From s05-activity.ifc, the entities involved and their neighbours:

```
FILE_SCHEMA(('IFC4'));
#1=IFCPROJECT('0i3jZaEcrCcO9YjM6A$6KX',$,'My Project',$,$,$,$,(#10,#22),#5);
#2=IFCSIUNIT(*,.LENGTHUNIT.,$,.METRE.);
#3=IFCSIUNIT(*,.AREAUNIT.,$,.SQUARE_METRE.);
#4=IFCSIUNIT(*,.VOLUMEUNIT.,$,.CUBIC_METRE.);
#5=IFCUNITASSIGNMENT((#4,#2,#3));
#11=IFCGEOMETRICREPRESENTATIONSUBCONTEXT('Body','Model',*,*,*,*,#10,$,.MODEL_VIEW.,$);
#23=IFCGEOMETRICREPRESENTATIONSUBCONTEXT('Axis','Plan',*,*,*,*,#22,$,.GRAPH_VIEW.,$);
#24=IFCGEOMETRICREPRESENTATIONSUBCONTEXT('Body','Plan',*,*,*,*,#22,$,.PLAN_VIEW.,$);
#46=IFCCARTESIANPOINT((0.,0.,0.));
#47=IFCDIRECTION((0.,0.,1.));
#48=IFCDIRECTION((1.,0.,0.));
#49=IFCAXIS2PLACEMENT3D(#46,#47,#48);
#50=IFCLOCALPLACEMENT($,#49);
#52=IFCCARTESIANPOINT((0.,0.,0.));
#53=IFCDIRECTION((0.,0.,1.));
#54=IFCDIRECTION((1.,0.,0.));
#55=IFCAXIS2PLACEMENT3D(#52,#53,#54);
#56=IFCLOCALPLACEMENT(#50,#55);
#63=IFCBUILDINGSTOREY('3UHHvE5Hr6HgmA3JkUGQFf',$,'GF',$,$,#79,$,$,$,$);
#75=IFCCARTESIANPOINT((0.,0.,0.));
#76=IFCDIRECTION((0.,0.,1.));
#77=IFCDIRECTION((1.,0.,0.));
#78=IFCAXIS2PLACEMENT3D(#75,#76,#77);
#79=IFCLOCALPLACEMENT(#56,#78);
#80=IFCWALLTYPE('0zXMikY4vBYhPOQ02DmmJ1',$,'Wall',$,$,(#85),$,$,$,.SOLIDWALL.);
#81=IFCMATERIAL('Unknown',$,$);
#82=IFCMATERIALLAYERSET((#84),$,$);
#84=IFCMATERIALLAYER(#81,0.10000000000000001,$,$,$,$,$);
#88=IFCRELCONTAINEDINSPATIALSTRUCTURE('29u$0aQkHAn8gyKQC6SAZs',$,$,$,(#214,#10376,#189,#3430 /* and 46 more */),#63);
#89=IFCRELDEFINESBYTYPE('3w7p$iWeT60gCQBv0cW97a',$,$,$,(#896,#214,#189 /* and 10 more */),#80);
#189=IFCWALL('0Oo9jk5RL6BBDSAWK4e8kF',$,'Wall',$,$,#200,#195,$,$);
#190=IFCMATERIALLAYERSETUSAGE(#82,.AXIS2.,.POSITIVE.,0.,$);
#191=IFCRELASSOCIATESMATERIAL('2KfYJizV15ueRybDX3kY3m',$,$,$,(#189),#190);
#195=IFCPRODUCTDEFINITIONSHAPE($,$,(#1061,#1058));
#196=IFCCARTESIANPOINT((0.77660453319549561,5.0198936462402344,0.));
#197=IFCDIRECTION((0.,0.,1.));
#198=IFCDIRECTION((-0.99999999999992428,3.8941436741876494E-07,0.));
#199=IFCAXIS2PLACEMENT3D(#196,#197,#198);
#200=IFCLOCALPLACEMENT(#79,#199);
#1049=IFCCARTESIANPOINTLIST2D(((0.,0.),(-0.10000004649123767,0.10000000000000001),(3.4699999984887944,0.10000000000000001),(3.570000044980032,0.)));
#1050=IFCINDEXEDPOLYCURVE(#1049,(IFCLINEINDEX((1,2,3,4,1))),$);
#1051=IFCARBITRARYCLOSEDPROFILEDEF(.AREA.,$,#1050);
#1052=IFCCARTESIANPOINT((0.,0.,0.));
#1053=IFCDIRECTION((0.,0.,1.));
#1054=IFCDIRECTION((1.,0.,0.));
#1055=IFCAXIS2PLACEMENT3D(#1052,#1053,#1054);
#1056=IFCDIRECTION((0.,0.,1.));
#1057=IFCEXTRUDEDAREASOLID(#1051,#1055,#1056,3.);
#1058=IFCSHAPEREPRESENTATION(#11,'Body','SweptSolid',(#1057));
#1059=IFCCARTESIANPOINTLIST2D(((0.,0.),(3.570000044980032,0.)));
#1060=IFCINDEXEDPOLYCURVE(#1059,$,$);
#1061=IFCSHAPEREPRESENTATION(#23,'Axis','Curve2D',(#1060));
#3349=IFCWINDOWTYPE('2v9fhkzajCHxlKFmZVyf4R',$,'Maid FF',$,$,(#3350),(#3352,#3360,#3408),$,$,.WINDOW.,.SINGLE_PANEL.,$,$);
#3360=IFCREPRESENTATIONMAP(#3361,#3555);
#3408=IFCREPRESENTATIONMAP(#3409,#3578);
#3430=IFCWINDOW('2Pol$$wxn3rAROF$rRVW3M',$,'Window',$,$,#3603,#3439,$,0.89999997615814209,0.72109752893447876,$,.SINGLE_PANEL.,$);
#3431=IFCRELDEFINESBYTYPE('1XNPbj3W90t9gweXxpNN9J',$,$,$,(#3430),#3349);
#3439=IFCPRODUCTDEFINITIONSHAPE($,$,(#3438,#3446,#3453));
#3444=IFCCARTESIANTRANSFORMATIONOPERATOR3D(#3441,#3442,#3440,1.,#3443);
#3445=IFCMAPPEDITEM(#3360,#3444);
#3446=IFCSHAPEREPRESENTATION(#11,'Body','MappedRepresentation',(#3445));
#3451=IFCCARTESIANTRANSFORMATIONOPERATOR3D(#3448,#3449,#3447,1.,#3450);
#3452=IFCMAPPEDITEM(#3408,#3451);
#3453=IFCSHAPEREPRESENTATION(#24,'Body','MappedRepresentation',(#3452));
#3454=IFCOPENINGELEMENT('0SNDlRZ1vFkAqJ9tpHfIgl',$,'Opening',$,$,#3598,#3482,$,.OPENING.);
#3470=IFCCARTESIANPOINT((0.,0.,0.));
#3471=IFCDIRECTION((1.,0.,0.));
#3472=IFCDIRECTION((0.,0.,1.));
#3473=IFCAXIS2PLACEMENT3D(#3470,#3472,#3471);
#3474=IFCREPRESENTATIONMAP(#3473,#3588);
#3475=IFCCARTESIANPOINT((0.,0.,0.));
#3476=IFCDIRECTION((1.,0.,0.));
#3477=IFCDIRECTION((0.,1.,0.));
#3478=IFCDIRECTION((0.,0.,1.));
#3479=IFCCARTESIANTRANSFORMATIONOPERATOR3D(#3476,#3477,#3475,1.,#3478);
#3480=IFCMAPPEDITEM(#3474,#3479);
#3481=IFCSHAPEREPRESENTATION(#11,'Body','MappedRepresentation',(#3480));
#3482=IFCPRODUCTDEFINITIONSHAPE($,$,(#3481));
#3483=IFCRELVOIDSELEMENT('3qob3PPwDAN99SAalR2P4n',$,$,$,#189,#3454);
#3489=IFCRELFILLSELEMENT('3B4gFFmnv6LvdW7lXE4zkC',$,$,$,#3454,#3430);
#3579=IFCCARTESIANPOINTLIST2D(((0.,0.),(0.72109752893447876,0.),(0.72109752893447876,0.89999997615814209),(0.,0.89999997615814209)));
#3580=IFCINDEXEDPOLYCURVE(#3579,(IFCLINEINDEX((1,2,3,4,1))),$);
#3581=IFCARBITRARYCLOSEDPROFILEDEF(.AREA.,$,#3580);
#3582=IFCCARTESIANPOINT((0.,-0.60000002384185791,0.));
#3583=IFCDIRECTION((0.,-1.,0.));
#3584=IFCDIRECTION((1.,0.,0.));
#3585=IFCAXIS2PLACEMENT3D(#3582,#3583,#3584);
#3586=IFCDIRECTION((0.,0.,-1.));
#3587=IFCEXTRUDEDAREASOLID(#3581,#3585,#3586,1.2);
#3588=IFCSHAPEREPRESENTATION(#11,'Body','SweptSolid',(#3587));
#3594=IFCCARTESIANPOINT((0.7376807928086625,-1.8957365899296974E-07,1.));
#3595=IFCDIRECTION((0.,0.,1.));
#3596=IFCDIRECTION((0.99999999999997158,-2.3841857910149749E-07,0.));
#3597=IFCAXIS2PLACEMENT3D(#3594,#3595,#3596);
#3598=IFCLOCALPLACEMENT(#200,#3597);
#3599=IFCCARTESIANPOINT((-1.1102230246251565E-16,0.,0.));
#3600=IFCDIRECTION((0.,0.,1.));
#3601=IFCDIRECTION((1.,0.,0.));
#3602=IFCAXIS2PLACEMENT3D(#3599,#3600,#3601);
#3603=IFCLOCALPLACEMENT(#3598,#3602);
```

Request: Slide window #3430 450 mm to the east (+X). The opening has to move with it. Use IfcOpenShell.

```python
import ifcopenshell
import ifcopenshell.api.geometry
import ifcopenshell.util.placement

model = ifcopenshell.open("s05-activity.ifc")

window = model.by_id(3430)
opening = window.FillsVoids[0].RelatingOpeningElement
wall = opening.VoidsElements[0].RelatingBuildingElement

wall_matrix = ifcopenshell.util.placement.get_local_placement(wall.ObjectPlacement)
shift = wall_matrix[:3, 0] * -0.45
before = ifcopenshell.util.placement.get_local_placement(window.ObjectPlacement)[:3, 3].copy()

# The window is placed relative to its opening, so it follows when the opening moves.
matrix = ifcopenshell.util.placement.get_local_placement(opening.ObjectPlacement)
matrix[:3, 3] += shift
ifcopenshell.api.geometry.edit_object_placement(
    model, product=opening, matrix=matrix, is_si=False, should_transform_children=True
)

after = ifcopenshell.util.placement.get_local_placement(window.ObjectPlacement)[:3, 3]
print("window moved by", (after - before).round(3) + 0.0)

model.write("s05-activity_updated.ifc")
```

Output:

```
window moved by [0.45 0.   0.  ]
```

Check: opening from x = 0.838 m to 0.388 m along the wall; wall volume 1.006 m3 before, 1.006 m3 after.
